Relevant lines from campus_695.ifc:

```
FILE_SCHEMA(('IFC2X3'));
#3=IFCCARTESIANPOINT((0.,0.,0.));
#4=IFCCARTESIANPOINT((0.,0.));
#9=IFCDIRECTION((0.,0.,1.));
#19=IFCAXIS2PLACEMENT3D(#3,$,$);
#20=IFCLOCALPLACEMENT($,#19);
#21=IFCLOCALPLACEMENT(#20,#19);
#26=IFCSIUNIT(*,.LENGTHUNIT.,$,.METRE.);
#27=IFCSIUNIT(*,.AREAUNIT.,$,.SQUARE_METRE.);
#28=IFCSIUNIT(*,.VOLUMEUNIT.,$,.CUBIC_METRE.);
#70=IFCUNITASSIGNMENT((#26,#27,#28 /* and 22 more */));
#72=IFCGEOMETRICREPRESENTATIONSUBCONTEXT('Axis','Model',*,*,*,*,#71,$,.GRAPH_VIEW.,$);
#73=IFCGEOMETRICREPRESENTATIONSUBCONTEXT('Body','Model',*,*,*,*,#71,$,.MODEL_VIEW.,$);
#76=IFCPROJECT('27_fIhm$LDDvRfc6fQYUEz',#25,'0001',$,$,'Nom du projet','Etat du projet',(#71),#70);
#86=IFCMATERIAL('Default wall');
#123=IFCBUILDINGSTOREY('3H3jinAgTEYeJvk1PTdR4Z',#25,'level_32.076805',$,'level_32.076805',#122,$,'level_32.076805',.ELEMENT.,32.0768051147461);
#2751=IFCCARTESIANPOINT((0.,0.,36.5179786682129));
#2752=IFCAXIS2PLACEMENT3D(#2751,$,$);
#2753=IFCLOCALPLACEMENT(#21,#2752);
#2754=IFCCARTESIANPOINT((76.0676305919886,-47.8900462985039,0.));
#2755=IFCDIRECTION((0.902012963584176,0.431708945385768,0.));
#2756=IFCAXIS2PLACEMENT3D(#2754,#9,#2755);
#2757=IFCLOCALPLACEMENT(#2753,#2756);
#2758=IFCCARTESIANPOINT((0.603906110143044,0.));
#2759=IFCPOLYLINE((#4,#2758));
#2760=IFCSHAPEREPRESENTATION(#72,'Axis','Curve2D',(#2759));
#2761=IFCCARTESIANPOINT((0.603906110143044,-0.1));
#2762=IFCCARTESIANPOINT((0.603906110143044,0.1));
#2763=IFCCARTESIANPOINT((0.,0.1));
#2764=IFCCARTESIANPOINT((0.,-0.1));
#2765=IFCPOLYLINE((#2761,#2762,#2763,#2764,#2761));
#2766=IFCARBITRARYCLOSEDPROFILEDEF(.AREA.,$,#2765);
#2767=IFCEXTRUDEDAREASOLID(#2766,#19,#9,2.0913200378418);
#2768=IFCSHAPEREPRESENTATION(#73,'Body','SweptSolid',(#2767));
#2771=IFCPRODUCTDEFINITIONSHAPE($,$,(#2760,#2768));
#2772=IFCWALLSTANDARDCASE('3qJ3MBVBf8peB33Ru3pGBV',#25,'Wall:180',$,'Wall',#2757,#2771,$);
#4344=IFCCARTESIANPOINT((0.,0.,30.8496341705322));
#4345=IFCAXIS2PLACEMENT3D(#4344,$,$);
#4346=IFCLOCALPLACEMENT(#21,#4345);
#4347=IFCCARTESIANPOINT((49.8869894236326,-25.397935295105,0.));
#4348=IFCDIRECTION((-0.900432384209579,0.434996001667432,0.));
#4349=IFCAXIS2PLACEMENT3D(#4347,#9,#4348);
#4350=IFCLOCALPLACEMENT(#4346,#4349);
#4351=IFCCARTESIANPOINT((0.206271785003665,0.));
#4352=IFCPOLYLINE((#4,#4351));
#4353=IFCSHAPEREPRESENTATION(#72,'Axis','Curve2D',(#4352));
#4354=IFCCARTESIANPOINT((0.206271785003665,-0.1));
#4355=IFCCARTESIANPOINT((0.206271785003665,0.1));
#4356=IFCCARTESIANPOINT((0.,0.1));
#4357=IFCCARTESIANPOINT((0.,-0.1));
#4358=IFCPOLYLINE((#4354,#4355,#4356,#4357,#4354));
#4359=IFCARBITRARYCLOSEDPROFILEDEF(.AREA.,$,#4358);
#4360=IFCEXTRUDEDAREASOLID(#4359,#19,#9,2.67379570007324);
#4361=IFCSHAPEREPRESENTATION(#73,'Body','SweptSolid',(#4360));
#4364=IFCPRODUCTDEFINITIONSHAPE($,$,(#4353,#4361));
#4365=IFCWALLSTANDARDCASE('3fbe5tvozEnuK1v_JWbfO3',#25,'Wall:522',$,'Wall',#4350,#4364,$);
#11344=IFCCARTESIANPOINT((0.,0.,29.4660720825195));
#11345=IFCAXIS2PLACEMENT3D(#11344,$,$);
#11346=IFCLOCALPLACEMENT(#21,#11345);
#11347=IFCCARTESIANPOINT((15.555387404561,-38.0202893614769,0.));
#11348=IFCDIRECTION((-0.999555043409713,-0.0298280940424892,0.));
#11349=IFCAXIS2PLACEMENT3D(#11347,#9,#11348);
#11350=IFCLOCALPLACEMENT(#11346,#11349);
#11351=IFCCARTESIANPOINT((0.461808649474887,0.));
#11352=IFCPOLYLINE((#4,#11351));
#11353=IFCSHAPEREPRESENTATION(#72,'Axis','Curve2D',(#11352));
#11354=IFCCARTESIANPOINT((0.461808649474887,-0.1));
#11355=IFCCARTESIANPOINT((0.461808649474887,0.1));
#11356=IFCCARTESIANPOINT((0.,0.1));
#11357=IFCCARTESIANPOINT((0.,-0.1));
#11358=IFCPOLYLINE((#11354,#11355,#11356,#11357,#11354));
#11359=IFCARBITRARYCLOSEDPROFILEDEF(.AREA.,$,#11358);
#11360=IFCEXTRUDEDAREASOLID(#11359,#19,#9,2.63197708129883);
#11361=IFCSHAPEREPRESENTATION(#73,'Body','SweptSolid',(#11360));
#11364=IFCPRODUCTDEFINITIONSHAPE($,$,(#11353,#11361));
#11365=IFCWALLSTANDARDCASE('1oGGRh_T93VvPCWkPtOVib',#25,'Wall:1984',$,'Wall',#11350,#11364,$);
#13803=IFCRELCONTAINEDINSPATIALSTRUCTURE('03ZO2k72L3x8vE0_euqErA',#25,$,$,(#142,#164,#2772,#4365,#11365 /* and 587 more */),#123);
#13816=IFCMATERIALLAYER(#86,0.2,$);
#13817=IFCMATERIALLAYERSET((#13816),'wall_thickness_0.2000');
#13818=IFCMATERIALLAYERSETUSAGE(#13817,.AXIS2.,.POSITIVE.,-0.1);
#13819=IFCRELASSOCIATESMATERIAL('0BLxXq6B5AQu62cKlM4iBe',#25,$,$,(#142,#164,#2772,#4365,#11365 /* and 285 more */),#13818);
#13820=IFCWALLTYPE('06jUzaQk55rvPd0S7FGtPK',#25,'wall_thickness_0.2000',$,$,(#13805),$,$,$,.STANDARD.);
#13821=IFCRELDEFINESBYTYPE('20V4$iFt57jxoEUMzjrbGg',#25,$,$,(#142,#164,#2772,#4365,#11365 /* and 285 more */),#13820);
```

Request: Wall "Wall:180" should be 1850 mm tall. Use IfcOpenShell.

```python
import ifcopenshell
import ifcopenshell.geom
import ifcopenshell.util.representation
import ifcopenshell.util.shape

model = ifcopenshell.open("campus_695.ifc")
settings = ifcopenshell.geom.settings()


def volume(element):
    """Net volume in cubic metres, openings subtracted."""
    shape = ifcopenshell.geom.create_shape(settings, element)
    return ifcopenshell.util.shape.get_volume(shape.geometry)


wall = model.by_guid("3qJ3MBVBf8peB33Ru3pGBV")
before = volume(wall)

body = ifcopenshell.util.representation.get_representation(wall, "Model", "Body")
solid = body.Items[0]
old_height = solid.Depth
solid.Depth = 1.85
after = volume(wall)

print(f"height {old_height:g} -> {solid.Depth:g}, volume {before:.3f} -> {after:.3f} m3")

model.write("campus_695_edited.ifc")
```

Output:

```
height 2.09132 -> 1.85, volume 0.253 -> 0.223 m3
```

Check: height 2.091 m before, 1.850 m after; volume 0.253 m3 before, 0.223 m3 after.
